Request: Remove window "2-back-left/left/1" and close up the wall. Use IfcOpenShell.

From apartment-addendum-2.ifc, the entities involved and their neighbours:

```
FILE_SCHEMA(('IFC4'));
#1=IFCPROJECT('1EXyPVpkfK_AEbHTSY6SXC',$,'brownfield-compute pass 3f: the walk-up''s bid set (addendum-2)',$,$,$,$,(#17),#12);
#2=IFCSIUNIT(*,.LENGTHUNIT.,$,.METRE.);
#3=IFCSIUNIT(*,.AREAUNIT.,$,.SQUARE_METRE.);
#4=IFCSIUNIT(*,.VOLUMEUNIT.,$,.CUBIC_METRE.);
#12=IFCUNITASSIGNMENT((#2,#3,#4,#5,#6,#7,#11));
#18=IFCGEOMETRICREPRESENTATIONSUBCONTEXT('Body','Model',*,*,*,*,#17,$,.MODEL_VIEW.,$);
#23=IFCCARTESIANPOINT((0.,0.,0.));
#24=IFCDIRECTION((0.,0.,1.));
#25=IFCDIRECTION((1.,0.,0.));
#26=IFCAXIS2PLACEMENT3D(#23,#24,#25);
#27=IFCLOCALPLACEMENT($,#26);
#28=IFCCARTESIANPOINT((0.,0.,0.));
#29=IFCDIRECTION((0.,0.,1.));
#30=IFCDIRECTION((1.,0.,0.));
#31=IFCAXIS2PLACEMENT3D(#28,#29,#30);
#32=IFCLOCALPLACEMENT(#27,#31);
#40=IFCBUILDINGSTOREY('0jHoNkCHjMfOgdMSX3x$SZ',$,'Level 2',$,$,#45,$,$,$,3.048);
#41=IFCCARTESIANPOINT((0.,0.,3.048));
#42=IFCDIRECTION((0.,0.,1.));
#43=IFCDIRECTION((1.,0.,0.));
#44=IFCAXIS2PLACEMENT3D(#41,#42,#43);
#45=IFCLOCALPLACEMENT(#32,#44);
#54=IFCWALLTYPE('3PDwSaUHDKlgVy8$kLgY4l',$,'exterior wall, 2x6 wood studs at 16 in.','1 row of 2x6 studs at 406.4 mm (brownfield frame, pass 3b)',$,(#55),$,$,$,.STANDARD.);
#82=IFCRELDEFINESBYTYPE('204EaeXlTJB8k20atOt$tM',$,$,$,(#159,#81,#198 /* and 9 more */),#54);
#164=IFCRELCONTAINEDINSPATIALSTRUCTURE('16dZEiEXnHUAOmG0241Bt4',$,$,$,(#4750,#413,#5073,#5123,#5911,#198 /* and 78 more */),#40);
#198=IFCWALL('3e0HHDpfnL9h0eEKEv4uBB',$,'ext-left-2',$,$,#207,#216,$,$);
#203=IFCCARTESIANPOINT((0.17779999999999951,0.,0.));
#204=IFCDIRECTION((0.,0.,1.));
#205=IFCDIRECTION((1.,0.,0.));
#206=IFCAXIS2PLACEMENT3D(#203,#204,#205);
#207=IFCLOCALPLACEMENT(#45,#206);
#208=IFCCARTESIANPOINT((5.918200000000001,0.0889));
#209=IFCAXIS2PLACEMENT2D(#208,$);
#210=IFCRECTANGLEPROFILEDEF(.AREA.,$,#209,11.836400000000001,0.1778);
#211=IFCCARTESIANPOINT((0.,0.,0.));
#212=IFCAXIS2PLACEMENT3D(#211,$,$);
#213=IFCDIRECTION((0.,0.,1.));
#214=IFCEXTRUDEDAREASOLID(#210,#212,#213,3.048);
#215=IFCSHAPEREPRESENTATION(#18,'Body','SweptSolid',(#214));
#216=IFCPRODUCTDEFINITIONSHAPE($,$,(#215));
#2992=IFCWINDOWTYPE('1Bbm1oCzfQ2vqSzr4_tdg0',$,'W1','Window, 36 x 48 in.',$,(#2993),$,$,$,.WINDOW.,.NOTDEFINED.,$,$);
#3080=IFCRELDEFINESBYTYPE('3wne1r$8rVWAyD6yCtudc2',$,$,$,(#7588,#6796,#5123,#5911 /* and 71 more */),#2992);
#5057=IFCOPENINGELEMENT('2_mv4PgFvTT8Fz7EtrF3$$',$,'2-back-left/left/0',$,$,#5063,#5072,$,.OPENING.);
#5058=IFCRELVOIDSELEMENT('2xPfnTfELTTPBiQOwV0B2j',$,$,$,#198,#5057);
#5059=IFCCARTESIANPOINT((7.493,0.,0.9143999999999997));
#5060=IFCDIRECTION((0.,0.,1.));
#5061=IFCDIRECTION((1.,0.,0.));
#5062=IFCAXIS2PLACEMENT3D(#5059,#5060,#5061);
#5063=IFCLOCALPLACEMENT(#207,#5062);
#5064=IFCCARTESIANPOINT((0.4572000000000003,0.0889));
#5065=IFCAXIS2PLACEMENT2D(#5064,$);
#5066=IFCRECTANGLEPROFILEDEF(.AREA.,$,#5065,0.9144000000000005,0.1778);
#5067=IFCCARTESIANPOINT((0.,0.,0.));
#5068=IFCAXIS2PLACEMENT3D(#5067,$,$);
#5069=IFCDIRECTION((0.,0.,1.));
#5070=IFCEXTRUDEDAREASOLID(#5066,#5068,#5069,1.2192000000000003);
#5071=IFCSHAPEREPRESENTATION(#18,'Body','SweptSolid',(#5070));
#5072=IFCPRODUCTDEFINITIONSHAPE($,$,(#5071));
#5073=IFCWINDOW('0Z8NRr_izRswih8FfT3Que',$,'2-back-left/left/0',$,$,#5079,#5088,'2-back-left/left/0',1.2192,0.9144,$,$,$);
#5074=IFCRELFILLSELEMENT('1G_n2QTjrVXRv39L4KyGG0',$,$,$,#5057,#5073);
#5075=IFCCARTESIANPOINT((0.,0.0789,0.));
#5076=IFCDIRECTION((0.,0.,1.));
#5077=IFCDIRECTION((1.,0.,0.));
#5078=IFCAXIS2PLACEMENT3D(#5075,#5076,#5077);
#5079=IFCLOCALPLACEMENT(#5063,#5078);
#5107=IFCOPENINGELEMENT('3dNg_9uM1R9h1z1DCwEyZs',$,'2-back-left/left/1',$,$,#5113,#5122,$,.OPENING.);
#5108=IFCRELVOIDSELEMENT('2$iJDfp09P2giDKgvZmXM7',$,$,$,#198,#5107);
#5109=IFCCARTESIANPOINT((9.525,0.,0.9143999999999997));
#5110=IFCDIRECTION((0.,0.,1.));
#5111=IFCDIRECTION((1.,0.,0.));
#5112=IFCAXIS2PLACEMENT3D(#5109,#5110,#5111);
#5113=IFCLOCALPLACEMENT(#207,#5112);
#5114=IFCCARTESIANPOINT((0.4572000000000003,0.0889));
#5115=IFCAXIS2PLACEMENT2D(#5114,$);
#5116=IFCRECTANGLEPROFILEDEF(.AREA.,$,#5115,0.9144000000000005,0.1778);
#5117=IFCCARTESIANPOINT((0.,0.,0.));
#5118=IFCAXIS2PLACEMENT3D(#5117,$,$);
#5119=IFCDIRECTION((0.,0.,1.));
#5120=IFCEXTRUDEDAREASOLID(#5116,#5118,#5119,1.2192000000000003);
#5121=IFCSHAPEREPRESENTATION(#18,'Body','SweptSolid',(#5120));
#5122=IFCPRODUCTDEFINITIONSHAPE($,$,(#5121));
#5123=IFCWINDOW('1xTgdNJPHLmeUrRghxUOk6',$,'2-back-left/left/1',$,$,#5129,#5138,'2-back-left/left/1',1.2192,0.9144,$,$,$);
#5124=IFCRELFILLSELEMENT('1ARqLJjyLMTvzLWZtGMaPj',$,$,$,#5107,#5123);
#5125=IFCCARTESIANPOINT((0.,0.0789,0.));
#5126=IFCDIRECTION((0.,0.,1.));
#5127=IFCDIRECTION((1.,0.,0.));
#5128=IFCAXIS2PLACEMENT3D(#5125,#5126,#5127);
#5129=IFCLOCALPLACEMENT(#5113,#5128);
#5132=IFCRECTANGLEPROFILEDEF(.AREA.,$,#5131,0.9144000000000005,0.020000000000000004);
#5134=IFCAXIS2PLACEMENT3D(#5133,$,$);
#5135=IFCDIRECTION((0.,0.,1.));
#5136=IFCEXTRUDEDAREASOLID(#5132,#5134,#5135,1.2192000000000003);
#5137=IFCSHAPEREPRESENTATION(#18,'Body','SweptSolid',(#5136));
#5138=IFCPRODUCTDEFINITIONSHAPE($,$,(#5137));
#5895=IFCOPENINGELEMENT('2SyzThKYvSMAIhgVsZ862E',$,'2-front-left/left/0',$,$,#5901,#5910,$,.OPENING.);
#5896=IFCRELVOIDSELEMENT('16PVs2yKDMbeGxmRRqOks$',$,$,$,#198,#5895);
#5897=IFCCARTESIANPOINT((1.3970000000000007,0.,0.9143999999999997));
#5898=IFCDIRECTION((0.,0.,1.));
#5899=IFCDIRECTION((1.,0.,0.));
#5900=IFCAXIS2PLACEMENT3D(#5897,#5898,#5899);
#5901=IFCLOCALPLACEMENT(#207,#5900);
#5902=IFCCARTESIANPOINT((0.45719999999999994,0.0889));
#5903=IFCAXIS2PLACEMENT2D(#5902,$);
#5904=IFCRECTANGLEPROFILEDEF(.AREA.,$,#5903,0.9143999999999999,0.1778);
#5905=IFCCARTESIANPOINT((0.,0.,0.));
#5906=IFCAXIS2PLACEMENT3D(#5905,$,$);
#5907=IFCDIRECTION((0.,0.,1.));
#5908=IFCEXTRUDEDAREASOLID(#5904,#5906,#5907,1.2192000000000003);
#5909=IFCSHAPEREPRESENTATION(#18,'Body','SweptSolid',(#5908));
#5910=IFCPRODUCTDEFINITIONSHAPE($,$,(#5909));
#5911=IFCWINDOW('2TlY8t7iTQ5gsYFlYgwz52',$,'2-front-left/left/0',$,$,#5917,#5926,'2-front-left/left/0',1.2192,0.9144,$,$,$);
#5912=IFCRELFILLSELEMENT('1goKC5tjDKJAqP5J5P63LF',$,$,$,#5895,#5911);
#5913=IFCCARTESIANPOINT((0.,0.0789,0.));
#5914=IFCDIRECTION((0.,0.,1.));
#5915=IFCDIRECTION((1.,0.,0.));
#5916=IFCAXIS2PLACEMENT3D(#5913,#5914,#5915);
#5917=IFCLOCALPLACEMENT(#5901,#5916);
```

```python
import ifcopenshell
import ifcopenshell.api.feature
import ifcopenshell.api.root
import ifcopenshell.geom
import ifcopenshell.util.shape

model = ifcopenshell.open("apartment-addendum-2.ifc")
settings = ifcopenshell.geom.settings()


def volume(element):
    """Net volume in cubic metres, openings subtracted."""
    shape = ifcopenshell.geom.create_shape(settings, element)
    return ifcopenshell.util.shape.get_volume(shape.geometry)


window = model.by_guid("1xTgdNJPHLmeUrRghxUOk6")
opening = window.FillsVoids[0].RelatingOpeningElement
wall = opening.VoidsElements[0].RelatingBuildingElement
before = volume(wall)

ifcopenshell.api.root.remove_product(model, product=window)
ifcopenshell.api.feature.remove_feature(model, feature=opening)

after = volume(wall)

print(f"wall volume {before:.3f} -> {after:.3f} m3")

model.write("apartment-addendum-2_updated.ifc")
```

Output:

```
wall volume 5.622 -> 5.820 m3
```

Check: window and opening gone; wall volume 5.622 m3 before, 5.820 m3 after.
